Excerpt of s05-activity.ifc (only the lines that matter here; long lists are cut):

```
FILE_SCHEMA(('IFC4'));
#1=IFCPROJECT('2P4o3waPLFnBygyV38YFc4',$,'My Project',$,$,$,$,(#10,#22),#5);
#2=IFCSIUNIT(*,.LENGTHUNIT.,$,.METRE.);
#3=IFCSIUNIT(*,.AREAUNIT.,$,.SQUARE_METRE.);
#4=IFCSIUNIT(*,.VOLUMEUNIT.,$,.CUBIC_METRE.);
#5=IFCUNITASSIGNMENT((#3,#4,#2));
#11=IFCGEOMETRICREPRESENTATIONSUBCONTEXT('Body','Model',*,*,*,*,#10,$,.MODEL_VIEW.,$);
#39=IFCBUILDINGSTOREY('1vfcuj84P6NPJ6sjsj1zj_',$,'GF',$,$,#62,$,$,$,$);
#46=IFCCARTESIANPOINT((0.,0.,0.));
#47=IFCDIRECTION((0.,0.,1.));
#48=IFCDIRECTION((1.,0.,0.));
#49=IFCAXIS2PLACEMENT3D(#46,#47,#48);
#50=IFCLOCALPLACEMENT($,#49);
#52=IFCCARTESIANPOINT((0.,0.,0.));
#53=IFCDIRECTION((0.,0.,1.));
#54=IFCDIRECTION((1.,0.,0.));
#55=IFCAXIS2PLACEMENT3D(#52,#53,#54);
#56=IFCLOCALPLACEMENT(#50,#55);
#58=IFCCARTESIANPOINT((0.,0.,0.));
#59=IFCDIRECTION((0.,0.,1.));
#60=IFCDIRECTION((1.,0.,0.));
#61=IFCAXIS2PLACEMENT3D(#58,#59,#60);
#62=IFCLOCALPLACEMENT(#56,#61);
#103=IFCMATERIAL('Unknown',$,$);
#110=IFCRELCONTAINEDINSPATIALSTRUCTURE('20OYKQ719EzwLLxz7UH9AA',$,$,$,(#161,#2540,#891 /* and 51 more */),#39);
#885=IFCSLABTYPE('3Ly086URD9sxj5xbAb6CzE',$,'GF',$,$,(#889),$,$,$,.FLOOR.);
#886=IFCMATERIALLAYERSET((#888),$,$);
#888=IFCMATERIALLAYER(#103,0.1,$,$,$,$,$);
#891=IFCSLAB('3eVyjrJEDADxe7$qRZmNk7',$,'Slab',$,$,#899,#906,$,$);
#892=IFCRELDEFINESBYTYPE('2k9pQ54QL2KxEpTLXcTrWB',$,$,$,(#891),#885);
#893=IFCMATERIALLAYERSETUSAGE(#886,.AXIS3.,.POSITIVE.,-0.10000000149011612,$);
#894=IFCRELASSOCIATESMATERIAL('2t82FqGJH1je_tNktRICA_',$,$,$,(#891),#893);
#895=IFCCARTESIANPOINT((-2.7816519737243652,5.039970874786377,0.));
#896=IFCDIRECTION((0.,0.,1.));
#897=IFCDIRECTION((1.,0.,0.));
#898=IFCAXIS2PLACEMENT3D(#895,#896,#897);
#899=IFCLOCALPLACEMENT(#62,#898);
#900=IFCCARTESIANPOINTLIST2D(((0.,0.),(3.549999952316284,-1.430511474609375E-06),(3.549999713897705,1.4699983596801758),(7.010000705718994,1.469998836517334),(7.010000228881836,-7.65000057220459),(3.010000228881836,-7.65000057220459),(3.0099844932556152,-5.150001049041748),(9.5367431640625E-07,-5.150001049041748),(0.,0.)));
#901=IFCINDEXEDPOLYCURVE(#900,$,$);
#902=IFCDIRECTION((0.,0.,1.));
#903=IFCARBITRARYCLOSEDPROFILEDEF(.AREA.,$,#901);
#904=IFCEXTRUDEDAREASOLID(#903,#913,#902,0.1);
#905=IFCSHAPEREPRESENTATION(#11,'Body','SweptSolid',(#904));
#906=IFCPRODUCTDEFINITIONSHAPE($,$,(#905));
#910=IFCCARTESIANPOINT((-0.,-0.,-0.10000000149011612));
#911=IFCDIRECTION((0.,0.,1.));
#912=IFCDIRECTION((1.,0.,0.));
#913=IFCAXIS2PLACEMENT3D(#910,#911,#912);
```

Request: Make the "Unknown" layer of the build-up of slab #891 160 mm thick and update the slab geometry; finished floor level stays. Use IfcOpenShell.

```python
import ifcopenshell
import ifcopenshell.util.element
import ifcopenshell.util.representation
import ifcopenshell.util.unit

model = ifcopenshell.open("s05-activity.ifc")
unit_scale = ifcopenshell.util.unit.calculate_unit_scale(model)

layer_set = model.by_id(886)
layer = next(l for l in layer_set.MaterialLayers if l.Material and l.Material.Name == "Unknown")
change = 0.16 / unit_scale - layer.LayerThickness
layer.LayerThickness += change

# Geometry does not follow the layer set by itself.
slabs = [e for e in ifcopenshell.util.element.get_elements_by_material(model, layer_set) if e.is_a("IfcSlab")]
for slab in sorted(slabs, key=lambda e: e.id()):
    body = ifcopenshell.util.representation.get_representation(slab, "Model", "Body")
    solid = body.Items[0]
    old_depth = solid.Depth
    solid.Depth += change
    # Extruded upwards: lower the start of the extrusion so the top stays.
    x, y, z = solid.Position.Location.Coordinates
    solid.Position.Location = model.createIfcCartesianPoint((x, y, z - change))
    print(slab.id(), f"{old_depth:g} -> {solid.Depth:g}")

# The layers are counted up from the underside, which has moved.
for usage in {ifcopenshell.util.element.get_material(slab) for slab in slabs}:
    usage.OffsetFromReferenceLine -= change

model.write("s05-activity_rev.ifc")
```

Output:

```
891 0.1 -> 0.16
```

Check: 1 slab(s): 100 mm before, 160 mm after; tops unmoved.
